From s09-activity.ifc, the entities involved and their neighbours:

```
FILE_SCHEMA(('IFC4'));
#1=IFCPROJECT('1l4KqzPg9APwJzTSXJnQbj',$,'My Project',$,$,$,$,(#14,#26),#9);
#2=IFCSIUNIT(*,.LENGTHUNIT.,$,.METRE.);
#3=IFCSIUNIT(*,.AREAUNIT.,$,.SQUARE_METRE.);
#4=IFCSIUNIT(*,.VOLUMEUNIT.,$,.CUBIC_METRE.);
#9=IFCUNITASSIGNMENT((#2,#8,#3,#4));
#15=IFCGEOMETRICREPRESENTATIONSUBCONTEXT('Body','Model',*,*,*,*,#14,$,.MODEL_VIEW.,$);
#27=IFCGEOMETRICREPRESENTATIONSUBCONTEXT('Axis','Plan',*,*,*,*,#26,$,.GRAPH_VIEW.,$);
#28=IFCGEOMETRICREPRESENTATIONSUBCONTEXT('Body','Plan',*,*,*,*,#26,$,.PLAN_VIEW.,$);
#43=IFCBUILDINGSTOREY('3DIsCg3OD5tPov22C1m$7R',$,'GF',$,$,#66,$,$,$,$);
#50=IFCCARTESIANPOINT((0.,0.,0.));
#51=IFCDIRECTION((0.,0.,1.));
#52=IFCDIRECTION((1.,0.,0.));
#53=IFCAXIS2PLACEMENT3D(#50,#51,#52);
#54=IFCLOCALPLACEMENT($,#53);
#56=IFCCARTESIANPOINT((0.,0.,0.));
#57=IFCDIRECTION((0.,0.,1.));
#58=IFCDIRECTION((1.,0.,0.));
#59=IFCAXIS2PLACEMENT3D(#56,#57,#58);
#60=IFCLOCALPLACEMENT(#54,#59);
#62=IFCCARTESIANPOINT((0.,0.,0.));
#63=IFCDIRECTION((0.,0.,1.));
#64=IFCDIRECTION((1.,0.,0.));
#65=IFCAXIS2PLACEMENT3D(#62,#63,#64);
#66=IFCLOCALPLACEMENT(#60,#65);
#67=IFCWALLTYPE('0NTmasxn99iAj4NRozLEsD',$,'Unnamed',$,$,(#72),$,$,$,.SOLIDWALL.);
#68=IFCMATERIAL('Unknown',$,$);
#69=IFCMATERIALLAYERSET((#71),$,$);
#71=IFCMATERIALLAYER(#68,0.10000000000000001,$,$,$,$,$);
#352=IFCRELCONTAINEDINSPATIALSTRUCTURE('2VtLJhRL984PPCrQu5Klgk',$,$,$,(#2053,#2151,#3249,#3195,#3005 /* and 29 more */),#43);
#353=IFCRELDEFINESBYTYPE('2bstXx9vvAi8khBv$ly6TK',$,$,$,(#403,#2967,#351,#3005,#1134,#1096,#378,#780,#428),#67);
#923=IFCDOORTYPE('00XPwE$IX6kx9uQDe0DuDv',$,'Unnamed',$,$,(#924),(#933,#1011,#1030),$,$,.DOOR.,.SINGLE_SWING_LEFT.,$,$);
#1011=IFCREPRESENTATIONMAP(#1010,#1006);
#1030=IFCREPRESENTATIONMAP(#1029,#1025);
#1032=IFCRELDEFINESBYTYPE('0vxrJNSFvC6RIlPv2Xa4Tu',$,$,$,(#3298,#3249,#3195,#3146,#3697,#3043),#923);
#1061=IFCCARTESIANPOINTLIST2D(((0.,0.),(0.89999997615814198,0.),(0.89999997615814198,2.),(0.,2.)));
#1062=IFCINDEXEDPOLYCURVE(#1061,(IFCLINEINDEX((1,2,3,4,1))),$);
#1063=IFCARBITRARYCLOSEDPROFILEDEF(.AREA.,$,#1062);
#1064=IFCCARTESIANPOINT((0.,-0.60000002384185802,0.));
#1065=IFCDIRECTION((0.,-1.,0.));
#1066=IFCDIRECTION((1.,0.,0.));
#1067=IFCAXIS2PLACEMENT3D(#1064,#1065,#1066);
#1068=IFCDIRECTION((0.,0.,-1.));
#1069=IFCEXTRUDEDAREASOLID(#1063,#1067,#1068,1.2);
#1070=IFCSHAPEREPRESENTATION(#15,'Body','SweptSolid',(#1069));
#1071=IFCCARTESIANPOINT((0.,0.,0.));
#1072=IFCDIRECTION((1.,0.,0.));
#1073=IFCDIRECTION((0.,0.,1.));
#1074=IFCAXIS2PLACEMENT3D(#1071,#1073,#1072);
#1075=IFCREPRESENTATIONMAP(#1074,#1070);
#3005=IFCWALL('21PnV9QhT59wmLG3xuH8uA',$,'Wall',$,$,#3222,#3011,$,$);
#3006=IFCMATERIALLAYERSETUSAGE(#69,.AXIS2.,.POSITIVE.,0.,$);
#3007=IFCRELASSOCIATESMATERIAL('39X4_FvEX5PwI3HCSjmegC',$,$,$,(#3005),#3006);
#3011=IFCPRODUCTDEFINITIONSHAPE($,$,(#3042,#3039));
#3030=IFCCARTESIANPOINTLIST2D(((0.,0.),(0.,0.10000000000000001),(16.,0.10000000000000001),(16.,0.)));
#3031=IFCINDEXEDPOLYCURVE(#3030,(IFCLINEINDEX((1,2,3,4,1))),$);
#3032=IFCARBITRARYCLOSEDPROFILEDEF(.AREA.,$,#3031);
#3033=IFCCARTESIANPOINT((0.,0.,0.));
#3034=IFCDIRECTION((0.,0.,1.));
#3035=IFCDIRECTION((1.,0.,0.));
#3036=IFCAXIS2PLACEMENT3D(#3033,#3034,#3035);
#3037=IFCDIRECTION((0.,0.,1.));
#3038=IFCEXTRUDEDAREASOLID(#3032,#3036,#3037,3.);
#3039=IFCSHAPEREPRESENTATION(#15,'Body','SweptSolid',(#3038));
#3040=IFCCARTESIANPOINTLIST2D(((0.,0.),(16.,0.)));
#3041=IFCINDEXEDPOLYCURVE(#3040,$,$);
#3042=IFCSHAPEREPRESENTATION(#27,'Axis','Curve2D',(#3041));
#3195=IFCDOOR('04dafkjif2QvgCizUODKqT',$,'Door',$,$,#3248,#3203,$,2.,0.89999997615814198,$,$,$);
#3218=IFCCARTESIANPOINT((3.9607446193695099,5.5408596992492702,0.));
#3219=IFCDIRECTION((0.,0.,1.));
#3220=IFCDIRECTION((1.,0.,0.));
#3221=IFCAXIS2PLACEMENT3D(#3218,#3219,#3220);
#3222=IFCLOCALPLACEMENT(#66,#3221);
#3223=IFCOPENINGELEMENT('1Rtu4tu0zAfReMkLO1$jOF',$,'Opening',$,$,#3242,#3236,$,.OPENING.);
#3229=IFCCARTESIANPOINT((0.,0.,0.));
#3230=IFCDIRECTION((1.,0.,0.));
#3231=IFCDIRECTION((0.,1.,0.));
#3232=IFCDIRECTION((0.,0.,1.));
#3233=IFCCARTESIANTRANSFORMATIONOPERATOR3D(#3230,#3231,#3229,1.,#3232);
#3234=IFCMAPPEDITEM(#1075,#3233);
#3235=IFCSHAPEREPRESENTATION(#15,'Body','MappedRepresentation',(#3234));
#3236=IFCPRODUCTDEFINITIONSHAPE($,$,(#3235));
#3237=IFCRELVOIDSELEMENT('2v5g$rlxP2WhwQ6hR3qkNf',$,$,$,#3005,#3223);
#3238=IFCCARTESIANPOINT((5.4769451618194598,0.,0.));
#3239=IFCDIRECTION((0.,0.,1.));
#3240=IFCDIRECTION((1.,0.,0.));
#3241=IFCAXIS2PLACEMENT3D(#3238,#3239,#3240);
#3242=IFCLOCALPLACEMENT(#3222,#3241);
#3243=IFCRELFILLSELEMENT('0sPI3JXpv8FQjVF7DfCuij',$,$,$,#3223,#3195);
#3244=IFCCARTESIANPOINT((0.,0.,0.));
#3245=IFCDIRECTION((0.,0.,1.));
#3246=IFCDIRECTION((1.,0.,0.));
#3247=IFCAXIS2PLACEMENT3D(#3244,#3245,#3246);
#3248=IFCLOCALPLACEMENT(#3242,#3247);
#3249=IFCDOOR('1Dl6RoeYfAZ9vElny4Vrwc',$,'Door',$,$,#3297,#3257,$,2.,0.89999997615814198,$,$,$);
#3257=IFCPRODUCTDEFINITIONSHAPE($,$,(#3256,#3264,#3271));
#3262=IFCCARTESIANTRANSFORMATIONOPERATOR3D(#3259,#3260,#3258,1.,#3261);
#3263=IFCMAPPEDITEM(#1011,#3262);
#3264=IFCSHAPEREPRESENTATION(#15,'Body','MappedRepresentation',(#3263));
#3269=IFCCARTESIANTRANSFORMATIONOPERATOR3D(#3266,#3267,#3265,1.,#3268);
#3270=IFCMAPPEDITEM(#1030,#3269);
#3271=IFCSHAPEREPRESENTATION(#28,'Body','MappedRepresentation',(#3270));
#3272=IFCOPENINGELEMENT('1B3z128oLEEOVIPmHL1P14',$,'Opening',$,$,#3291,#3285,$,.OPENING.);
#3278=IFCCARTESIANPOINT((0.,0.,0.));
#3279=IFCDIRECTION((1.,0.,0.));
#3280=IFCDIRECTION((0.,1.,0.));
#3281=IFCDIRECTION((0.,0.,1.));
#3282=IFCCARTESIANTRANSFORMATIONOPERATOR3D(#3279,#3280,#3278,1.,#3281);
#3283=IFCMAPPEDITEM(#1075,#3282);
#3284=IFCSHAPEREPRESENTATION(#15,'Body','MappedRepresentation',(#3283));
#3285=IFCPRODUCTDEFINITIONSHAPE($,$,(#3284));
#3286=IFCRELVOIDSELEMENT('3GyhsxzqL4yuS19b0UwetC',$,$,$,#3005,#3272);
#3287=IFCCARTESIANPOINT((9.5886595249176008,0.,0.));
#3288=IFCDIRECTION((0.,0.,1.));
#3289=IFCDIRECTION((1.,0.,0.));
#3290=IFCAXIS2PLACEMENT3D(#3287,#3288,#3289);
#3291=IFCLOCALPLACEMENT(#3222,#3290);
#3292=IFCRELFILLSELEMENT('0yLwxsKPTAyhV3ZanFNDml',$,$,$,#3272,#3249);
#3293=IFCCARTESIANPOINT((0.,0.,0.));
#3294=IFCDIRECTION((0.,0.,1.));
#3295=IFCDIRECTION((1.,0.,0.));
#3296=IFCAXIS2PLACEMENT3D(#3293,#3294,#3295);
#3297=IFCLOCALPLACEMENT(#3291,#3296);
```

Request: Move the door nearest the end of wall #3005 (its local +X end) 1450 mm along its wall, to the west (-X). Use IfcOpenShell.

```python
import ifcopenshell
import ifcopenshell.api.geometry
import ifcopenshell.util.placement

model = ifcopenshell.open("s09-activity.ifc")

door = model.by_id(3249)
opening = door.FillsVoids[0].RelatingOpeningElement
wall = opening.VoidsElements[0].RelatingBuildingElement

wall_matrix = ifcopenshell.util.placement.get_local_placement(wall.ObjectPlacement)
shift = wall_matrix[:3, 0] * -1.45
before = ifcopenshell.util.placement.get_local_placement(door.ObjectPlacement)[:3, 3].copy()

# The door is placed relative to its opening, so it follows when the opening moves.
matrix = ifcopenshell.util.placement.get_local_placement(opening.ObjectPlacement)
matrix[:3, 3] += shift
ifcopenshell.api.geometry.edit_object_placement(
    model, product=opening, matrix=matrix, is_si=False, should_transform_children=True
)

after = ifcopenshell.util.placement.get_local_placement(door.ObjectPlacement)[:3, 3]
print("door moved by", (after - before).round(3) + 0.0)

model.write("s09-activity_rev.ifc")
```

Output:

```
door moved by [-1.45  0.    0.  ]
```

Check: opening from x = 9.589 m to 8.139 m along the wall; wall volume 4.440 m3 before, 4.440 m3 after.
